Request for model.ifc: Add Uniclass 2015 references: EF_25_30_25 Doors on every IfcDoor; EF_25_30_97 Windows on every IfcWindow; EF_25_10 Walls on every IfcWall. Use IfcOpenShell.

First a look at what the model holds.

```python
import ifcopenshell

model = ifcopenshell.open("model.ifc")
print(model.schema)
print("classifications:", [c.Name for c in model.by_type("IfcClassification")])
for ifc_class in ("IfcDoor", "IfcRoof", "IfcStair", "IfcWall", "IfcWindow"):
    print(ifc_class, len(model.by_type(ifc_class)))
```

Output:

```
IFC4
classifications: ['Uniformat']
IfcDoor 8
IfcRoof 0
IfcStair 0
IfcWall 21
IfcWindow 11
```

```python
import ifcopenshell
import ifcopenshell.api.classification

model = ifcopenshell.open("model.ifc")

system = ifcopenshell.api.classification.add_classification(model, classification="Uniclass 2015")

codes = {
    "IfcDoor": ("EF_25_30_25", "Doors"),
    "IfcWindow": ("EF_25_30_97", "Windows"),
    "IfcWall": ("EF_25_10", "Walls"),
}
for ifc_class, (code, name) in codes.items():
    products = model.by_type(ifc_class)
    ifcopenshell.api.classification.add_reference(
        model, products=products, classification=system, identification=code, name=name
    )
    print(code, len(products))

model.write("model_updated.ifc")
```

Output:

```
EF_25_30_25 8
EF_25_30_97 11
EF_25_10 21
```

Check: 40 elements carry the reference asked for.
